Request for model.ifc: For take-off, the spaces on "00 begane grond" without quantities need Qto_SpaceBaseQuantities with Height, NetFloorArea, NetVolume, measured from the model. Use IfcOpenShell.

First a look at what the model holds.

```python
import ifcopenshell
import ifcopenshell.util.element
import ifcopenshell.util.unit

model = ifcopenshell.open("model.ifc")
print(model.schema)
for unit_type in ("LENGTHUNIT", "AREAUNIT", "VOLUMEUNIT"):
    print(unit_type, ifcopenshell.util.unit.calculate_unit_scale(model, unit_type))
storey = next(s for s in model.by_type("IfcBuildingStorey") if s.Name == "00 begane grond")
spaces = [e for e in ifcopenshell.util.element.get_decomposition(storey) if e.is_a("IfcSpace")]
for e in sorted(spaces, key=lambda e: e.id()):
    print(e.id(), e.is_a(), e.Name, list(ifcopenshell.util.element.get_psets(e, qtos_only=True)), sep=" | ")
```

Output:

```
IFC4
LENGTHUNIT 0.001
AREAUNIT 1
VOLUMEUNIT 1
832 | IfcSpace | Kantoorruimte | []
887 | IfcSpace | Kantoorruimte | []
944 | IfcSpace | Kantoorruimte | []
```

```python
import ifcopenshell
import ifcopenshell.api.pset
import ifcopenshell.geom
import ifcopenshell.util.element
import ifcopenshell.util.shape
import ifcopenshell.util.unit

model = ifcopenshell.open("model.ifc")
unit_scale = ifcopenshell.util.unit.calculate_unit_scale(model)
area_scale = ifcopenshell.util.unit.calculate_unit_scale(model, "AREAUNIT")
volume_scale = ifcopenshell.util.unit.calculate_unit_scale(model, "VOLUMEUNIT")
settings = ifcopenshell.geom.settings()

storey = next(s for s in model.by_type("IfcBuildingStorey") if s.Name == "00 begane grond")
spaces = [e for e in ifcopenshell.util.element.get_decomposition(storey) if e.is_a("IfcSpace")]

for e in sorted(spaces, key=lambda e: e.id()):
    if ifcopenshell.util.element.get_psets(e, qtos_only=True, should_inherit=False):
        continue
    # Geometry comes back in metres, in the element's own axes.
    shape = ifcopenshell.geom.create_shape(settings, e)
    values = {
        "Height": ifcopenshell.util.shape.get_z(shape.geometry) / unit_scale,
        "NetFloorArea": ifcopenshell.util.shape.get_footprint_area(shape.geometry) / area_scale,
        "NetVolume": ifcopenshell.util.shape.get_volume(shape.geometry) / volume_scale,
    }
    qto = ifcopenshell.api.pset.add_qto(model, product=e, name="Qto_SpaceBaseQuantities")
    ifcopenshell.api.pset.edit_qto(model, qto=qto, properties=values)
    print(e.id(), {k: round(v, 3) for k, v in values.items()})

model.write("model_v2.ifc")
```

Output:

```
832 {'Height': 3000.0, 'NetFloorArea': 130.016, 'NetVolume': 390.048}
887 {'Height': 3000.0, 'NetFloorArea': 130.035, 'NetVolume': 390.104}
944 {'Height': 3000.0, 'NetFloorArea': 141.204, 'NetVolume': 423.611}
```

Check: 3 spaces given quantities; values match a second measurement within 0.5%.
